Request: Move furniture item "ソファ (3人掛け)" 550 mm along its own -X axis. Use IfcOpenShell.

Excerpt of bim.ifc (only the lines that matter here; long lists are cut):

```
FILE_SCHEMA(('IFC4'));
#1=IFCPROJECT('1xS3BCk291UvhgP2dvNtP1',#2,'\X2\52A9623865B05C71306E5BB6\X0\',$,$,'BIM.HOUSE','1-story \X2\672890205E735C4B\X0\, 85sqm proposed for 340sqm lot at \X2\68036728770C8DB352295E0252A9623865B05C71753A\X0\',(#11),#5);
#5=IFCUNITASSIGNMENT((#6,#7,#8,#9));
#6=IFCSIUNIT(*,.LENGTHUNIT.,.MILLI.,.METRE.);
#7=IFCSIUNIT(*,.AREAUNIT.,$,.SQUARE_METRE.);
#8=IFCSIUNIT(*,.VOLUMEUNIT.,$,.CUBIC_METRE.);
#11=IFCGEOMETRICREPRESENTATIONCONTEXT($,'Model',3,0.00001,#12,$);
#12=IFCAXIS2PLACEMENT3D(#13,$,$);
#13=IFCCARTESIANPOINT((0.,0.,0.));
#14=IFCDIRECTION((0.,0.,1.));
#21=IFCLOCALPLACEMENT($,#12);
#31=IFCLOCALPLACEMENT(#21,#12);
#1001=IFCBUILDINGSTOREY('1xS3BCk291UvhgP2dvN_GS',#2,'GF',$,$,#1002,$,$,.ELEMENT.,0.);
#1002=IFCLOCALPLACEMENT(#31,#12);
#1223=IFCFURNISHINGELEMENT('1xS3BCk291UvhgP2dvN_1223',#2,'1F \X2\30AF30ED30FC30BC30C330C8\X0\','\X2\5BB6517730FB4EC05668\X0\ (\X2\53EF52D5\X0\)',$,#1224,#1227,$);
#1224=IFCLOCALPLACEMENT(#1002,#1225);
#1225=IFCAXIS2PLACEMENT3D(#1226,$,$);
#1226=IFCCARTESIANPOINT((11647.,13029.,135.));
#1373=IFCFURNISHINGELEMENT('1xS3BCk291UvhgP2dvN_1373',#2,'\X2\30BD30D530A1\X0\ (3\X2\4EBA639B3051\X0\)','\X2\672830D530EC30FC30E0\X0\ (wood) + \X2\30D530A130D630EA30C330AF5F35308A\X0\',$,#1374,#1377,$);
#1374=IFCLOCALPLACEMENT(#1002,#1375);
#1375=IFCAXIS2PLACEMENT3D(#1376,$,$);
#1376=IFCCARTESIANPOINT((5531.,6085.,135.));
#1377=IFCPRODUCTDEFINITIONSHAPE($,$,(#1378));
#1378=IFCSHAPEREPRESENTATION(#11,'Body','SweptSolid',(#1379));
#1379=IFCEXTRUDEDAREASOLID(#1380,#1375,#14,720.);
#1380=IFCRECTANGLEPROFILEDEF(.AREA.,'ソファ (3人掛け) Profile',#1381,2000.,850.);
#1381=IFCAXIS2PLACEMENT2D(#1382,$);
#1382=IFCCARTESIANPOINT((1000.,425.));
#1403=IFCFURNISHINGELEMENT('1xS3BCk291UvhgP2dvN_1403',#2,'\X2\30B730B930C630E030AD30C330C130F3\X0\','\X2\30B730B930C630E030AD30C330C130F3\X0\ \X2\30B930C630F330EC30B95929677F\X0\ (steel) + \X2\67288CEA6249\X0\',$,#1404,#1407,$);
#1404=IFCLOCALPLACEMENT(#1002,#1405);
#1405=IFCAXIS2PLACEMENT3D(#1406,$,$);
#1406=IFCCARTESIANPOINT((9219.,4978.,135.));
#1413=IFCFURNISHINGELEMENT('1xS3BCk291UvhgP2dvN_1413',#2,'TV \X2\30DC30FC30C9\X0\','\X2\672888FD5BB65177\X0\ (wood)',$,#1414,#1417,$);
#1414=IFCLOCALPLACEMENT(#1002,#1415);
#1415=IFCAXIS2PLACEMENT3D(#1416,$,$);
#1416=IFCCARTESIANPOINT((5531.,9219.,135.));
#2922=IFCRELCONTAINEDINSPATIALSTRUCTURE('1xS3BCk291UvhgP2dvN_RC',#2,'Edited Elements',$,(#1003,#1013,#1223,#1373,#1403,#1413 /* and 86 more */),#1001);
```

```python
import ifcopenshell
import ifcopenshell.api.geometry
import ifcopenshell.util.placement
import ifcopenshell.util.unit

model = ifcopenshell.open("bim.ifc")
unit_scale = ifcopenshell.util.unit.calculate_unit_scale(model)

item = model.by_id(1373)
matrix = ifcopenshell.util.placement.get_local_placement(item.ObjectPlacement)
matrix[:3, 3] -= matrix[:3, 0] * 0.55 / unit_scale
ifcopenshell.api.geometry.edit_object_placement(model, product=item, matrix=matrix, is_si=False)

print(ifcopenshell.util.placement.get_local_placement(item.ObjectPlacement).round(3) + 0.0)

model.write("bim-out.ifc")
```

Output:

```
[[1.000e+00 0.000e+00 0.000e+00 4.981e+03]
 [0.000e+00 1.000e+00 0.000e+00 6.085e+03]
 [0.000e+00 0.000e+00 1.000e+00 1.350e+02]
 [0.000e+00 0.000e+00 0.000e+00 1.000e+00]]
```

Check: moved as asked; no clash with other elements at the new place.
